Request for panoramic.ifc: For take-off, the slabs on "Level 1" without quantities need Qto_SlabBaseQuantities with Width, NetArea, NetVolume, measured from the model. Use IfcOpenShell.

First a look at what the model holds.

```python
import ifcopenshell
import ifcopenshell.util.element
import ifcopenshell.util.unit

model = ifcopenshell.open("panoramic.ifc")
print(model.schema)
for unit_type in ("LENGTHUNIT", "AREAUNIT", "VOLUMEUNIT"):
    print(unit_type, ifcopenshell.util.unit.calculate_unit_scale(model, unit_type))
storey = next(s for s in model.by_type("IfcBuildingStorey") if s.Name == "Level 1")
slabs = [e for e in ifcopenshell.util.element.get_decomposition(storey) if e.is_a("IfcSlab")]
for e in sorted(slabs, key=lambda e: e.id()):
    print(e.id(), e.is_a(), e.Name, list(ifcopenshell.util.element.get_psets(e, qtos_only=True)), sep=" | ")
```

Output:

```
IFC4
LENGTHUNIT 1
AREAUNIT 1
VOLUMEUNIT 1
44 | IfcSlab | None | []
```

```python
import ifcopenshell
import ifcopenshell.api.pset
import ifcopenshell.geom
import ifcopenshell.util.element
import ifcopenshell.util.shape
import ifcopenshell.util.unit

model = ifcopenshell.open("panoramic.ifc")
unit_scale = ifcopenshell.util.unit.calculate_unit_scale(model)
area_scale = ifcopenshell.util.unit.calculate_unit_scale(model, "AREAUNIT")
volume_scale = ifcopenshell.util.unit.calculate_unit_scale(model, "VOLUMEUNIT")
settings = ifcopenshell.geom.settings()

storey = next(s for s in model.by_type("IfcBuildingStorey") if s.Name == "Level 1")
slabs = [e for e in ifcopenshell.util.element.get_decomposition(storey) if e.is_a("IfcSlab")]

for e in sorted(slabs, key=lambda e: e.id()):
    if ifcopenshell.util.element.get_psets(e, qtos_only=True, should_inherit=False):
        continue
    # Geometry comes back in metres, in the element's own axes.
    shape = ifcopenshell.geom.create_shape(settings, e)
    values = {
        "Width": ifcopenshell.util.shape.get_z(shape.geometry) / unit_scale,
        "NetArea": ifcopenshell.util.shape.get_footprint_area(shape.geometry) / area_scale,
        "NetVolume": ifcopenshell.util.shape.get_volume(shape.geometry) / volume_scale,
    }
    qto = ifcopenshell.api.pset.add_qto(model, product=e, name="Qto_SlabBaseQuantities")
    ifcopenshell.api.pset.edit_qto(model, qto=qto, properties=values)
    print(e.id(), {k: round(v, 3) for k, v in values.items()})

model.write("panoramic_updated.ifc")
```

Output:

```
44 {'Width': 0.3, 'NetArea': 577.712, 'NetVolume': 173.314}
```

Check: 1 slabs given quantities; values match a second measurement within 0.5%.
